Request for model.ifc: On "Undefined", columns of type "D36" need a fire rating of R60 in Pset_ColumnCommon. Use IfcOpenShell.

First a look at what the model holds.

```python
import ifcopenshell
import ifcopenshell.util.element

model = ifcopenshell.open("model.ifc")
print(model.schema)
storey = next(s for s in model.by_type("IfcBuildingStorey") if s.Name == "Undefined")
columns = [e for e in ifcopenshell.util.element.get_decomposition(storey) if e.is_a("IfcColumn")]
seen = {}
for e in columns:
    element_type = ifcopenshell.util.element.get_type(e)
    key = (element_type.Name if element_type != e and element_type else None, ifcopenshell.util.element.get_pset(e, "Pset_ColumnCommon", "FireRating"))
    seen[key] = seen.get(key, 0) + 1
for (name, value), count in sorted(seen.items(), key=str):
    print(count, "x", name, "|", value)
```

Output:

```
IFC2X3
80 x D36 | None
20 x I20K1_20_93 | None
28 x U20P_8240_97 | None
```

```python
import ifcopenshell
import ifcopenshell.api.pset
import ifcopenshell.util.element

model = ifcopenshell.open("model.ifc")

storey = next(s for s in model.by_type("IfcBuildingStorey") if s.Name == "Undefined")
columns = [e for e in ifcopenshell.util.element.get_decomposition(storey) if e.is_a("IfcColumn")]

count = 0
for e in columns:
    element_type = ifcopenshell.util.element.get_type(e)
    if element_type in (None, e) or element_type.Name != "D36":
        continue
    found = ifcopenshell.util.element.get_pset(e, "Pset_ColumnCommon", should_inherit=False)
    if found:
        pset = model.by_id(found["id"])
        if len(ifcopenshell.util.element.get_elements_by_pset(pset)) > 1:
            pset = ifcopenshell.api.pset.unshare_pset(model, products=[e], pset=pset)[0]
    else:
        pset = ifcopenshell.api.pset.add_pset(model, product=e, name="Pset_ColumnCommon")
    ifcopenshell.api.pset.edit_pset(model, pset=pset, properties={"FireRating": "R60"})
    count += 1

print(count, "columns updated")

model.write("model_edited.ifc")
```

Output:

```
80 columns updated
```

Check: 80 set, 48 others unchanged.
